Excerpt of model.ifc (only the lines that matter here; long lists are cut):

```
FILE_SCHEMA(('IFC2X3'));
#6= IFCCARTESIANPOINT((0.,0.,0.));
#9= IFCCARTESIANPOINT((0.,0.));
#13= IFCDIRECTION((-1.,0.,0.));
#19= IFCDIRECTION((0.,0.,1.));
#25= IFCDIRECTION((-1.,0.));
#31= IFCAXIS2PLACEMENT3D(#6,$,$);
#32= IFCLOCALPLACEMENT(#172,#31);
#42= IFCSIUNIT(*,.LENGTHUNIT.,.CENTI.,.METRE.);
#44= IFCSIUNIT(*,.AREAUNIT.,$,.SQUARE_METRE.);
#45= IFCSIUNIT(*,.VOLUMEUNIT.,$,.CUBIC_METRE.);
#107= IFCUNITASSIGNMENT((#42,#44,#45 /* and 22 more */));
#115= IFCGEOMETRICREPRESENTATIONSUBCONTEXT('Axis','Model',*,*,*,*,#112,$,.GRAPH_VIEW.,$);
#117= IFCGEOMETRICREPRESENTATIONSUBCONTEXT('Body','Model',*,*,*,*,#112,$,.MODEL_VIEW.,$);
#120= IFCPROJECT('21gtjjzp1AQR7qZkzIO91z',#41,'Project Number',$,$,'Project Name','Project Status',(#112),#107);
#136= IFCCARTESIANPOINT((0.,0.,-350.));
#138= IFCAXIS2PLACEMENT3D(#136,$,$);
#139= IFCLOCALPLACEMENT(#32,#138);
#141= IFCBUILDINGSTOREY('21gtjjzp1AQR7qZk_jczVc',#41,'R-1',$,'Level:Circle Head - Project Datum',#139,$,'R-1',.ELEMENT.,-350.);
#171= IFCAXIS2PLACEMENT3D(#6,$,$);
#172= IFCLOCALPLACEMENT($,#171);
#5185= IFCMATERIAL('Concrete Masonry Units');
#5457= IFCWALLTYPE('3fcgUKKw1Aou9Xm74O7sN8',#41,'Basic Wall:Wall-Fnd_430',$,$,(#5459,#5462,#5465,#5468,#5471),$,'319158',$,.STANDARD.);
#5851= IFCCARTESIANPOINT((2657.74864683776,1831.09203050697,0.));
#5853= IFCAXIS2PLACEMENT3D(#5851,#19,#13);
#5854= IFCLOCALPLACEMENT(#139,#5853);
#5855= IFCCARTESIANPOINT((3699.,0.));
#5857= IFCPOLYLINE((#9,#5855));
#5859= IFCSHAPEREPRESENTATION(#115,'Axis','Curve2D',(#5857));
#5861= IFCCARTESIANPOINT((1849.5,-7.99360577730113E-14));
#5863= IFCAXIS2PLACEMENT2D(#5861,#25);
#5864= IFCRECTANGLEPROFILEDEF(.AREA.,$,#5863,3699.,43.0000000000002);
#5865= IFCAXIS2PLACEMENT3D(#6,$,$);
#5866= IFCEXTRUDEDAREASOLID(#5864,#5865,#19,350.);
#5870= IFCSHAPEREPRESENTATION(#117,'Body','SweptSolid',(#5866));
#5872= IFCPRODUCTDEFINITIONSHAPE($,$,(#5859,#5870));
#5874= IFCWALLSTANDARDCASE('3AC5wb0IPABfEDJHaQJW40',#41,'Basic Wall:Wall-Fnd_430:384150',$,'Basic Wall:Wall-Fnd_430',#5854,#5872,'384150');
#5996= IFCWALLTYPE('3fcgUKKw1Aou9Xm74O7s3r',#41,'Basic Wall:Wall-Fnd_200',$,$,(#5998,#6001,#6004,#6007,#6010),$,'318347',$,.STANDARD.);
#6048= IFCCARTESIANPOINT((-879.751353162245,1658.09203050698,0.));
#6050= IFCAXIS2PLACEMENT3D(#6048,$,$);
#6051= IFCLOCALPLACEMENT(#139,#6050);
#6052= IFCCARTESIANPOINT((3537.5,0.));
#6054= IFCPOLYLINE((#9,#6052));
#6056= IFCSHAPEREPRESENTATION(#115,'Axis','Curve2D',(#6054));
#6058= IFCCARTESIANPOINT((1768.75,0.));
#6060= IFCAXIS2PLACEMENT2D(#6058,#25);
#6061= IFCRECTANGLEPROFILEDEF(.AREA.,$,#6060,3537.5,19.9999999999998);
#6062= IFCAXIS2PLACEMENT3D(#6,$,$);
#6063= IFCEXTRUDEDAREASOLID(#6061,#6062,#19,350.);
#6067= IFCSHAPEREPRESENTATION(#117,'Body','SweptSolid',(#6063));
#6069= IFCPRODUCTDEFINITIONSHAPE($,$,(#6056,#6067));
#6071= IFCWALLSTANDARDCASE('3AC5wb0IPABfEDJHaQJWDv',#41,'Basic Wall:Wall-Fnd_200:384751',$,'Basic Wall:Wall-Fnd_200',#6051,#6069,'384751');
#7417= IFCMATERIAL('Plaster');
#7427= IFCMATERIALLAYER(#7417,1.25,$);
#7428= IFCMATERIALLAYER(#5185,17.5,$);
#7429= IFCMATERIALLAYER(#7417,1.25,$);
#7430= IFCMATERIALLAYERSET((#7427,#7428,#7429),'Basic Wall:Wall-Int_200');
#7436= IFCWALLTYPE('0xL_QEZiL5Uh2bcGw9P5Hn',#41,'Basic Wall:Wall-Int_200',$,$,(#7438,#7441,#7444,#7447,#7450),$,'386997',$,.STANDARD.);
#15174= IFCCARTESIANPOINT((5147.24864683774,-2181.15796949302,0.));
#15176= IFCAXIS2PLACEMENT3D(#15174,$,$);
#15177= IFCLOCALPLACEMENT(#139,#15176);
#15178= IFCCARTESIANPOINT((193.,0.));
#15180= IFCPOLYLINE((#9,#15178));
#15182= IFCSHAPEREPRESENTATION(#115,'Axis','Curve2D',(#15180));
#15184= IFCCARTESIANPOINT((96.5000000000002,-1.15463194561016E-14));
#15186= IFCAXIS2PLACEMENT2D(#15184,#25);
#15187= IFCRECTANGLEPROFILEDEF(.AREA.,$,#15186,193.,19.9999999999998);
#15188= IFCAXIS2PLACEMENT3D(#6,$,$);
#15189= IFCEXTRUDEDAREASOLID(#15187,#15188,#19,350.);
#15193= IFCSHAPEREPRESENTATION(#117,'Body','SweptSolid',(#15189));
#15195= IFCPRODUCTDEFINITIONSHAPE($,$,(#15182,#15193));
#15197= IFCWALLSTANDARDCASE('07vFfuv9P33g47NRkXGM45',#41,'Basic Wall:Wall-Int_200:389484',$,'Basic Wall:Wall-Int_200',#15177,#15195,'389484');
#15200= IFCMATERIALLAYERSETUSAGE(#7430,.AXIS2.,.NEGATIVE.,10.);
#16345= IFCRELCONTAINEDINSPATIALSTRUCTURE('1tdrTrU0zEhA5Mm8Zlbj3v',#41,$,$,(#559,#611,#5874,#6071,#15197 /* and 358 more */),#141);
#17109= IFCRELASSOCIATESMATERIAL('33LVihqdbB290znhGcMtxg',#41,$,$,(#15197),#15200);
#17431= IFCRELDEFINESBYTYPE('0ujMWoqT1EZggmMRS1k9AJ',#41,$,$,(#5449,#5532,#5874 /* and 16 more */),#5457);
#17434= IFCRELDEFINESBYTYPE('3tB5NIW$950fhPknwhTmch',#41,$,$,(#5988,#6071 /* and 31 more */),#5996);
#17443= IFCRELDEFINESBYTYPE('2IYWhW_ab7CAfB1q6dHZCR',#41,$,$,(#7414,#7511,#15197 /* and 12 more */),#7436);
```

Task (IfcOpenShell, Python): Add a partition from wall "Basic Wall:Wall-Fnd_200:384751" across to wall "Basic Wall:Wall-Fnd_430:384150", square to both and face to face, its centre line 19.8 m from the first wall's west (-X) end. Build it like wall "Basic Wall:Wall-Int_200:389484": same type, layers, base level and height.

```python
import numpy as np
import ifcopenshell
import ifcopenshell.api.geometry
import ifcopenshell.api.material
import ifcopenshell.api.pset
import ifcopenshell.api.root
import ifcopenshell.api.spatial
import ifcopenshell.api.type
import ifcopenshell.geom
import ifcopenshell.util.element
import ifcopenshell.util.placement
import ifcopenshell.util.representation
import ifcopenshell.util.shape
import ifcopenshell.util.unit

model = ifcopenshell.open("model.ifc")
unit_scale = ifcopenshell.util.unit.calculate_unit_scale(model)
settings = ifcopenshell.geom.settings()
settings.set("use-world-coords", True)

start_wall = model.by_id(6071)
end_wall = model.by_guid("3AC5wb0IPABfEDJHaQJW40")
like = model.by_guid("07vFfuv9P33g47NRkXGM45")
matrix = ifcopenshell.util.placement.get_local_placement(start_wall.ObjectPlacement)
matrix[:3, 3] *= unit_scale


def extent(element):
    """Bounding box in the first wall's axes, in metres."""
    shape = ifcopenshell.geom.create_shape(settings, element)
    points = (ifcopenshell.util.shape.get_vertices(shape.geometry) - matrix[:3, 3]) @ matrix[:3, :3]
    return points.min(axis=0), points.max(axis=0)


y_start = extent(start_wall)[1][1]
y_end = extent(end_wall)[0][1]
like_min, like_max = extent(like)
length, height = float(abs(y_end - y_start)), float(like_max[2] - like_min[2])
layer_set = ifcopenshell.util.element.get_material(like, should_skip_usage=True)
thickness = sum(layer.LayerThickness for layer in layer_set.MaterialLayers) * unit_scale

wall = ifcopenshell.api.root.create_entity(model, ifc_class="IfcWallStandardCase", name="New partition")
storey = ifcopenshell.util.element.get_container(like)
ifcopenshell.api.spatial.assign_container(model, products=[wall], relating_structure=storey)
ifcopenshell.api.type.assign_type(
    model, related_objects=[wall], relating_type=ifcopenshell.util.element.get_type(like), should_map_representations=False
)
rel = ifcopenshell.api.material.assign_material(
    model, products=[wall], type="IfcMaterialLayerSetUsage", material=layer_set
)
rel.RelatingMaterial.OffsetFromReferenceLine = -thickness / 2 / unit_scale
pset = ifcopenshell.api.pset.add_pset(model, product=wall, name="Pset_WallCommon")
ifcopenshell.api.pset.edit_pset(model, pset=pset, properties={"IsExternal": False, "LoadBearing": False})

# The axis runs down the middle of the wall.
axis = ifcopenshell.api.geometry.add_axis_representation(
    model, context=ifcopenshell.util.representation.get_context(model, "Model", "Axis"), axis=[(0.0, 0.0), (length, 0.0)]
)
body = ifcopenshell.api.geometry.add_wall_representation(
    model,
    context=ifcopenshell.util.representation.get_context(model, "Model", "Body", "MODEL_VIEW"),
    length=length,
    height=height,
    thickness=thickness,
    offset=-thickness / 2,
)
for representation in (axis, body):
    ifcopenshell.api.geometry.assign_representation(model, product=wall, representation=representation)

placement = matrix @ ifcopenshell.util.placement.rotation(90, "Z")
placement[:, 3] = matrix @ np.array([extent(start_wall)[0][0] + 19.8, y_start, like_min[2], 1.0])
ifcopenshell.api.geometry.edit_object_placement(model, product=wall, matrix=placement)

print(f"partition {length:.3f} m long, {height:.3f} m high, {thickness:.3f} m thick")

model.write("model_edited.ifc")
```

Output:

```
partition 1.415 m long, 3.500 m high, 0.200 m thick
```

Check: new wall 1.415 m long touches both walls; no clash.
